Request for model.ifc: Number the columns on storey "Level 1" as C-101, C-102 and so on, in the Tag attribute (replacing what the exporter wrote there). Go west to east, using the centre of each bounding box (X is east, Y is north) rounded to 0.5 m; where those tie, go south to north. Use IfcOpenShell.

First a look at what the model holds.

```python
import ifcopenshell
import ifcopenshell.util.element
import ifcopenshell.util.placement

model = ifcopenshell.open("model.ifc")
print(model.schema)
storey = next(s for s in model.by_type("IfcBuildingStorey") if s.Name == "Level 1")
columns = [e for e in ifcopenshell.util.element.get_decomposition(storey) if e.is_a("IfcColumn")]
for e in sorted(columns, key=lambda e: e.id()):
    origin = ifcopenshell.util.placement.get_local_placement(e.ObjectPlacement)[:3, 3]
    print(e.id(), e.Tag, e.Name, origin.round(2) + 0.0, sep=" | ")
```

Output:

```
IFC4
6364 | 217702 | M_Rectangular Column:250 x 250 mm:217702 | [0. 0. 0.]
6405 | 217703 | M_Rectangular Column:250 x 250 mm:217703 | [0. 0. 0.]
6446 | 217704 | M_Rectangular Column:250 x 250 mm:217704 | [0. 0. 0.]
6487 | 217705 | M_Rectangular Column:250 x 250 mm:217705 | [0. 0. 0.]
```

```python
import ifcopenshell
import ifcopenshell.geom
import ifcopenshell.util.element
import ifcopenshell.util.shape

model = ifcopenshell.open("model.ifc")
settings = ifcopenshell.geom.settings()
settings.set("use-world-coords", True)


def centre(element):
    shape = ifcopenshell.geom.create_shape(settings, element)
    return ifcopenshell.util.shape.get_bbox_centroid(shape.geometry)


storey = next(s for s in model.by_type("IfcBuildingStorey") if s.Name == "Level 1")
columns = [e for e in ifcopenshell.util.element.get_decomposition(storey) if e.is_a("IfcColumn")]

# Insertion points can sit at a corner or the storey origin, so sort by the geometry (in metres).
centres = {e: centre(e) for e in columns}
columns.sort(key=lambda e: (round(centres[e][0] / 0.5), centres[e][1]))

for i, e in enumerate(columns, start=1):
    number = f"C-1{i:02d}"
    e.Tag = number
    print(e.id(), number)

model.write("model_edited.ifc")
```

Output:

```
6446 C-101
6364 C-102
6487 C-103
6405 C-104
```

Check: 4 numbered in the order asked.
